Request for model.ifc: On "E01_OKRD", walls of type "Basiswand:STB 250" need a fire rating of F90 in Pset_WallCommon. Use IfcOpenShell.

First a look at what the model holds.

```python
import ifcopenshell
import ifcopenshell.util.element

model = ifcopenshell.open("model.ifc")
print(model.schema)
storey = next(s for s in model.by_type("IfcBuildingStorey") if s.Name == "E01_OKRD")
walls = [e for e in ifcopenshell.util.element.get_decomposition(storey) if e.is_a("IfcWall")]
seen = {}
for e in walls:
    element_type = ifcopenshell.util.element.get_type(e)
    key = (element_type.Name if element_type != e and element_type else None, ifcopenshell.util.element.get_pset(e, "Pset_WallCommon", "FireRating"))
    seen[key] = seen.get(key, 0) + 1
for (name, value), count in sorted(seen.items(), key=str):
    print(count, "x", name, "|", value)
```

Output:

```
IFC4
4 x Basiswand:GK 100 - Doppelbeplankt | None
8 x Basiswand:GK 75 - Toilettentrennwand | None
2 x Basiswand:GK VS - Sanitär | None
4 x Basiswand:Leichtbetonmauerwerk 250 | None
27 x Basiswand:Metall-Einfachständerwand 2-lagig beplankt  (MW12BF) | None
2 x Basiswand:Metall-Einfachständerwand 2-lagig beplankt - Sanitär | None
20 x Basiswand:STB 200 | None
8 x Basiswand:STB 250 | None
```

```python
import ifcopenshell
import ifcopenshell.api.pset
import ifcopenshell.util.element

model = ifcopenshell.open("model.ifc")

storey = next(s for s in model.by_type("IfcBuildingStorey") if s.Name == "E01_OKRD")
walls = [e for e in ifcopenshell.util.element.get_decomposition(storey) if e.is_a("IfcWall")]

count = 0
for e in walls:
    element_type = ifcopenshell.util.element.get_type(e)
    if element_type in (None, e) or element_type.Name != "Basiswand:STB 250":
        continue
    # add_pset returns the element's existing set when there is one.
    pset = ifcopenshell.api.pset.add_pset(model, product=e, name="Pset_WallCommon")
    ifcopenshell.api.pset.edit_pset(model, pset=pset, properties={"FireRating": "F90"})
    count += 1

print(count, "walls updated")

model.write("model-out.ifc")
```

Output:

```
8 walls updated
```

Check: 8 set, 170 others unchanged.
